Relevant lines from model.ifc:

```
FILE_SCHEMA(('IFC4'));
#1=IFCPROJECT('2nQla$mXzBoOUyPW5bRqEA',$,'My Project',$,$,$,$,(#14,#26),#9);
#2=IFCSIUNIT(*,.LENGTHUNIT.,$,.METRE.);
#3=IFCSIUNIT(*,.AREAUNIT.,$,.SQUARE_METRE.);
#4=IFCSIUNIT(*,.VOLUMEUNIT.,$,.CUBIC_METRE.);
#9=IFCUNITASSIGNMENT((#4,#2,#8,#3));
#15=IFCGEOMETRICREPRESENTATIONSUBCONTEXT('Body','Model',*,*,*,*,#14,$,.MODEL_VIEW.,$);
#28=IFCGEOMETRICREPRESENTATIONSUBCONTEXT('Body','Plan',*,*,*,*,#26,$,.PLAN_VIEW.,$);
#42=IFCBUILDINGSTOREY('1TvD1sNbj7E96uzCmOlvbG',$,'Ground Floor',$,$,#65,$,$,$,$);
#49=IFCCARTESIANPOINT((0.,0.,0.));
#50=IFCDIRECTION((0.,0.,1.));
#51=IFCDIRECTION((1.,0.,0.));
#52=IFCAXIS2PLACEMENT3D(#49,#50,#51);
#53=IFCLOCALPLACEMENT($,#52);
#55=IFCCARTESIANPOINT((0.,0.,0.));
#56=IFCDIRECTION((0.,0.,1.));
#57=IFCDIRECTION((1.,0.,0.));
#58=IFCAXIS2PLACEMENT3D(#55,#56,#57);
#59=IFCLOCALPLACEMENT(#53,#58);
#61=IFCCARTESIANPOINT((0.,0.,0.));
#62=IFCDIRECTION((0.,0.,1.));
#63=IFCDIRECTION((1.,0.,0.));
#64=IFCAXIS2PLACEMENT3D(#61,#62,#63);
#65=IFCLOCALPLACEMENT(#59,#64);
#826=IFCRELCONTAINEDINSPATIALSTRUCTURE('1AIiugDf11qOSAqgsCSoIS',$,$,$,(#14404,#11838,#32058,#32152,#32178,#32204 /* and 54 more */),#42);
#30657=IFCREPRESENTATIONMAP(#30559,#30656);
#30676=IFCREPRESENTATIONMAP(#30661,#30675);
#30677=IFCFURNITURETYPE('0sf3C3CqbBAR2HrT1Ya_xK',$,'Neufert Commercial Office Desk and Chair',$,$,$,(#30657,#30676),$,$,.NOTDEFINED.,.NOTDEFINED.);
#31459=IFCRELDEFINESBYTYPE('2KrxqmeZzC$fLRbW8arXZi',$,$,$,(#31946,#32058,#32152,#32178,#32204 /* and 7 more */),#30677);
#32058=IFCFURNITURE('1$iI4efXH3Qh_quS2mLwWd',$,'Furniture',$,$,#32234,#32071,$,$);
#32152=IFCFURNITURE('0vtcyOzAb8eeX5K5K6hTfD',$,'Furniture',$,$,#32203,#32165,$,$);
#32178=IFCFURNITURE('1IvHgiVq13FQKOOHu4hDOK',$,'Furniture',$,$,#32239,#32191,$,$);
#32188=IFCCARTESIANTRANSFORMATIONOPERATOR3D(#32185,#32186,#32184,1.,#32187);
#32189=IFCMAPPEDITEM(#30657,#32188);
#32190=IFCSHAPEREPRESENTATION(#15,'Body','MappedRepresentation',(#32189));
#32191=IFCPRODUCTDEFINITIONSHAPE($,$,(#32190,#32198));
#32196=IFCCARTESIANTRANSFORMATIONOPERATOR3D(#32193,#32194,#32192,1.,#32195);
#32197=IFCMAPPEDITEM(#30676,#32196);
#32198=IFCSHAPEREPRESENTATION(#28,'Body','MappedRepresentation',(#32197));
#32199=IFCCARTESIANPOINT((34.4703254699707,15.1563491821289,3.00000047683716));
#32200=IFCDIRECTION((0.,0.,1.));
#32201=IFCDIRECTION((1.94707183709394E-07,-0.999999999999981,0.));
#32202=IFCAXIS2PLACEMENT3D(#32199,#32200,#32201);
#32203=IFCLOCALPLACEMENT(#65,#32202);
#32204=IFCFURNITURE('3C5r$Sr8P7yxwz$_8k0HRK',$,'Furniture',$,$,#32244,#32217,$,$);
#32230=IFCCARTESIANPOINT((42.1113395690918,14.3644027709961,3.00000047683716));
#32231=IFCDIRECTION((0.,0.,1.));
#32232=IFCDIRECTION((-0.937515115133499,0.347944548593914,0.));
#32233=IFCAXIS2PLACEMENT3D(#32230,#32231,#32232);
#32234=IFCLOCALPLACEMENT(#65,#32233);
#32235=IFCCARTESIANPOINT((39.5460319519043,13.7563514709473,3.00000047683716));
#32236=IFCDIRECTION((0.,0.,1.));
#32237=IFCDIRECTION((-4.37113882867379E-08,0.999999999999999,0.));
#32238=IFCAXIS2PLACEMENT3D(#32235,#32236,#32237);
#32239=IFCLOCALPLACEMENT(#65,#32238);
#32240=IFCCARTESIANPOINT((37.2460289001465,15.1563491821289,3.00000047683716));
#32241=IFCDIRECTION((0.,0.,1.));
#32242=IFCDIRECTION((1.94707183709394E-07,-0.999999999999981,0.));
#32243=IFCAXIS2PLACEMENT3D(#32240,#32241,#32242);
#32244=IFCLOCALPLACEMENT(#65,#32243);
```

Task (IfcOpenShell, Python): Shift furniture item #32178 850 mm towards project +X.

```python
import ifcopenshell
import ifcopenshell.api.geometry
import ifcopenshell.util.placement
import ifcopenshell.util.unit

model = ifcopenshell.open("model.ifc")
unit_scale = ifcopenshell.util.unit.calculate_unit_scale(model)

item = model.by_guid("1IvHgiVq13FQKOOHu4hDOK")
matrix = ifcopenshell.util.placement.get_local_placement(item.ObjectPlacement)
matrix[0, 3] += 0.85 / unit_scale
ifcopenshell.api.geometry.edit_object_placement(model, product=item, matrix=matrix, is_si=False)

print(ifcopenshell.util.placement.get_local_placement(item.ObjectPlacement).round(3) + 0.0)

model.write("model-out.ifc")
```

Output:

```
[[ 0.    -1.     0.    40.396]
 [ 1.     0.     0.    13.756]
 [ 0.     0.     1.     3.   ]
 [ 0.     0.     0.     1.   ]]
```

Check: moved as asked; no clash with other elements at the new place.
